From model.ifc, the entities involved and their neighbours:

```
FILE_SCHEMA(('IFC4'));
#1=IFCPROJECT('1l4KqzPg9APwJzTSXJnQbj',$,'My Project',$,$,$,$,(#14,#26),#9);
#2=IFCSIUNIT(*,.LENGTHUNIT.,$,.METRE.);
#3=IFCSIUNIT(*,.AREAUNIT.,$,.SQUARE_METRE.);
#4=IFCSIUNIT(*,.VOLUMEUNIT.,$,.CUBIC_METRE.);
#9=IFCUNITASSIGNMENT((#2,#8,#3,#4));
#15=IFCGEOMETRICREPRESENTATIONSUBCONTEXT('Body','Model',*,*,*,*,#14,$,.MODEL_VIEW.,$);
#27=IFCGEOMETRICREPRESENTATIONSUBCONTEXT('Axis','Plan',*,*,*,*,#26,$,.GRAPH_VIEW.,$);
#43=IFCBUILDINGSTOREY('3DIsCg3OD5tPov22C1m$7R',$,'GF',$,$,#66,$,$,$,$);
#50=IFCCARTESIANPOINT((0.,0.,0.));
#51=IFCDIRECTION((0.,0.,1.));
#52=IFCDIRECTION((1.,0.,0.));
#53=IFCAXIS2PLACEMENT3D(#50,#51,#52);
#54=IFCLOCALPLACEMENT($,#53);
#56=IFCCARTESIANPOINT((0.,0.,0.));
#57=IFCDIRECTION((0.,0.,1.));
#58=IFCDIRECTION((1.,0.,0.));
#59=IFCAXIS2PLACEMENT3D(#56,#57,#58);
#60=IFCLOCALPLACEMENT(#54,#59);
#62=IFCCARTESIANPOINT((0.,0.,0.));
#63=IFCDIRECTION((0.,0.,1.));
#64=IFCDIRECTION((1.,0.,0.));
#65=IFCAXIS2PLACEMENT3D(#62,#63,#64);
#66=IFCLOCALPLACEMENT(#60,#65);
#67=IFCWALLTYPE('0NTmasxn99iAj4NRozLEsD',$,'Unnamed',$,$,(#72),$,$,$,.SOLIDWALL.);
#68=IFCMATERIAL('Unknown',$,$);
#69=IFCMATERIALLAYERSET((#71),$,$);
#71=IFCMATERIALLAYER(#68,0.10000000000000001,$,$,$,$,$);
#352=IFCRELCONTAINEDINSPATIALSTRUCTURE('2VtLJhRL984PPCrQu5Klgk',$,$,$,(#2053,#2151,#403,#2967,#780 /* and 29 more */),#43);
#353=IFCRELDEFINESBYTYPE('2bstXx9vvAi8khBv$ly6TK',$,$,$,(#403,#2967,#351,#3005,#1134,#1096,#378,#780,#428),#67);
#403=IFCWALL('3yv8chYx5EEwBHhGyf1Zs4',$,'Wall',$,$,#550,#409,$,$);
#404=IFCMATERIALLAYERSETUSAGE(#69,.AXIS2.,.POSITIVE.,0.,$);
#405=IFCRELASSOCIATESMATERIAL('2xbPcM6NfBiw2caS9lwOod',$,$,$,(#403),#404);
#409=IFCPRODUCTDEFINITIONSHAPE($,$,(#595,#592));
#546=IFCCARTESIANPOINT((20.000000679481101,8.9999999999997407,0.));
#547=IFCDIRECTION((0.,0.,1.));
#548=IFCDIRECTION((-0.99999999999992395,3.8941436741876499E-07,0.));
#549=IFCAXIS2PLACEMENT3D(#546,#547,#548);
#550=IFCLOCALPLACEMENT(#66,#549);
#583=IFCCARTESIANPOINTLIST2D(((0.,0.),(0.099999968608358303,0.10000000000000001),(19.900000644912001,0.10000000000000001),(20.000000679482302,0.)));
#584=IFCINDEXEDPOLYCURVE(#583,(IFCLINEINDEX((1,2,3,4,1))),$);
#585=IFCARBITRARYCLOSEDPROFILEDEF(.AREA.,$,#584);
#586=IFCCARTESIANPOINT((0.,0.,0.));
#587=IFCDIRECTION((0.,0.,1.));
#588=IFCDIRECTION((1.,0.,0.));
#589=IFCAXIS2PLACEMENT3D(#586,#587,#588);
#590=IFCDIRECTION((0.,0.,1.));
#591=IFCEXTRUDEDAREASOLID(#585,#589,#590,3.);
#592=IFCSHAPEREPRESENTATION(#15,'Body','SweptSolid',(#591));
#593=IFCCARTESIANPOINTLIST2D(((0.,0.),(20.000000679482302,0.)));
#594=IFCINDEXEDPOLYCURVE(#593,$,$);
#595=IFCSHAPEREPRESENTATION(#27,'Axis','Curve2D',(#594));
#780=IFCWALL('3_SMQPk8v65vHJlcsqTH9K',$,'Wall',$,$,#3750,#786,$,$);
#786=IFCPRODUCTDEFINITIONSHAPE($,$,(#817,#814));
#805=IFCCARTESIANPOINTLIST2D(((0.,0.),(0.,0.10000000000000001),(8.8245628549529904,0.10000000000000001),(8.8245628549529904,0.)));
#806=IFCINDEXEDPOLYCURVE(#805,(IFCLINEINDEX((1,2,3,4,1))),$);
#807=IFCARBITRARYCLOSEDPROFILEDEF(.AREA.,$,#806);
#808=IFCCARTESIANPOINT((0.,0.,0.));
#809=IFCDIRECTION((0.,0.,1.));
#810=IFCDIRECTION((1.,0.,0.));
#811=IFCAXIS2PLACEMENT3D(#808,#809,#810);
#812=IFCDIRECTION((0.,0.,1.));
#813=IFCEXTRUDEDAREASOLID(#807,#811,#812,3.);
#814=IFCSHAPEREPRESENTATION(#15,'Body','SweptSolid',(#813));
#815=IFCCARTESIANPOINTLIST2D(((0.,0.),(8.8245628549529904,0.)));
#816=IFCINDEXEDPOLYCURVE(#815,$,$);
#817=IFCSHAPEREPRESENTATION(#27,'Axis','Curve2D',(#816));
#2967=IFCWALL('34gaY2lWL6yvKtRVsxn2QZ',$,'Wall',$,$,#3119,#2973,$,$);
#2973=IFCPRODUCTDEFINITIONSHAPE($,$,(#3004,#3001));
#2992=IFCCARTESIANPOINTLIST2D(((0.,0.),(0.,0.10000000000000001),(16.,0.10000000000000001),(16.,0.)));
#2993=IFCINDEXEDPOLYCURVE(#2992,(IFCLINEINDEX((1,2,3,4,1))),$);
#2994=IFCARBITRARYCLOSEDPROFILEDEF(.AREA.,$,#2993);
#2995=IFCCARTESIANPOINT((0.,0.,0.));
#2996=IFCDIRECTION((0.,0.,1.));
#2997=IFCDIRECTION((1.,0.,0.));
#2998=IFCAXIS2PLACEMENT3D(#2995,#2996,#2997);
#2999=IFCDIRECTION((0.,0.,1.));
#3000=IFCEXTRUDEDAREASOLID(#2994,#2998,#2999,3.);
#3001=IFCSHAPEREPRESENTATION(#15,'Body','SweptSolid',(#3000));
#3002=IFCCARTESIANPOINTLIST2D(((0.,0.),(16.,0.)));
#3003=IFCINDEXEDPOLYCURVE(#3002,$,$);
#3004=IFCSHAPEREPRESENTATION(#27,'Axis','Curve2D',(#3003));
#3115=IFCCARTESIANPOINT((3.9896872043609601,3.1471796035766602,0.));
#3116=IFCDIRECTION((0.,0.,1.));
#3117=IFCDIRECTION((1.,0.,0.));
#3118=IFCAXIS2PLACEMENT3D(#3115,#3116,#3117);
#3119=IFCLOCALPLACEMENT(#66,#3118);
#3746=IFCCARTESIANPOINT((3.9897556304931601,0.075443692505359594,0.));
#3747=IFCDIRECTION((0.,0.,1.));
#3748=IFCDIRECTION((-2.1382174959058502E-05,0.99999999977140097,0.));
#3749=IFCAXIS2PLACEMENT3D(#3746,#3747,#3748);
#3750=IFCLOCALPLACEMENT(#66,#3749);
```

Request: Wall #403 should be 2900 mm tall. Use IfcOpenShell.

```python
import ifcopenshell
import ifcopenshell.geom
import ifcopenshell.util.representation
import ifcopenshell.util.shape
import ifcopenshell.util.unit

model = ifcopenshell.open("model.ifc")
unit_scale = ifcopenshell.util.unit.calculate_unit_scale(model)
settings = ifcopenshell.geom.settings()


def volume(element):
    """Net volume in cubic metres, openings subtracted."""
    shape = ifcopenshell.geom.create_shape(settings, element)
    return ifcopenshell.util.shape.get_volume(shape.geometry)


wall = model.by_guid("3yv8chYx5EEwBHhGyf1Zs4")
before = volume(wall)

body = ifcopenshell.util.representation.get_representation(wall, "Model", "Body")
solid = body.Items[0]
old_height = solid.Depth
solid.Depth = 2.9 / unit_scale
after = volume(wall)

print(f"height {old_height:g} -> {solid.Depth:g}, volume {before:.3f} -> {after:.3f} m3")

model.write("model_v2.ifc")
```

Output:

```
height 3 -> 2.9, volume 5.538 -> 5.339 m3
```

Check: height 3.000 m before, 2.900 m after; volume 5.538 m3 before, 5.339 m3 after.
